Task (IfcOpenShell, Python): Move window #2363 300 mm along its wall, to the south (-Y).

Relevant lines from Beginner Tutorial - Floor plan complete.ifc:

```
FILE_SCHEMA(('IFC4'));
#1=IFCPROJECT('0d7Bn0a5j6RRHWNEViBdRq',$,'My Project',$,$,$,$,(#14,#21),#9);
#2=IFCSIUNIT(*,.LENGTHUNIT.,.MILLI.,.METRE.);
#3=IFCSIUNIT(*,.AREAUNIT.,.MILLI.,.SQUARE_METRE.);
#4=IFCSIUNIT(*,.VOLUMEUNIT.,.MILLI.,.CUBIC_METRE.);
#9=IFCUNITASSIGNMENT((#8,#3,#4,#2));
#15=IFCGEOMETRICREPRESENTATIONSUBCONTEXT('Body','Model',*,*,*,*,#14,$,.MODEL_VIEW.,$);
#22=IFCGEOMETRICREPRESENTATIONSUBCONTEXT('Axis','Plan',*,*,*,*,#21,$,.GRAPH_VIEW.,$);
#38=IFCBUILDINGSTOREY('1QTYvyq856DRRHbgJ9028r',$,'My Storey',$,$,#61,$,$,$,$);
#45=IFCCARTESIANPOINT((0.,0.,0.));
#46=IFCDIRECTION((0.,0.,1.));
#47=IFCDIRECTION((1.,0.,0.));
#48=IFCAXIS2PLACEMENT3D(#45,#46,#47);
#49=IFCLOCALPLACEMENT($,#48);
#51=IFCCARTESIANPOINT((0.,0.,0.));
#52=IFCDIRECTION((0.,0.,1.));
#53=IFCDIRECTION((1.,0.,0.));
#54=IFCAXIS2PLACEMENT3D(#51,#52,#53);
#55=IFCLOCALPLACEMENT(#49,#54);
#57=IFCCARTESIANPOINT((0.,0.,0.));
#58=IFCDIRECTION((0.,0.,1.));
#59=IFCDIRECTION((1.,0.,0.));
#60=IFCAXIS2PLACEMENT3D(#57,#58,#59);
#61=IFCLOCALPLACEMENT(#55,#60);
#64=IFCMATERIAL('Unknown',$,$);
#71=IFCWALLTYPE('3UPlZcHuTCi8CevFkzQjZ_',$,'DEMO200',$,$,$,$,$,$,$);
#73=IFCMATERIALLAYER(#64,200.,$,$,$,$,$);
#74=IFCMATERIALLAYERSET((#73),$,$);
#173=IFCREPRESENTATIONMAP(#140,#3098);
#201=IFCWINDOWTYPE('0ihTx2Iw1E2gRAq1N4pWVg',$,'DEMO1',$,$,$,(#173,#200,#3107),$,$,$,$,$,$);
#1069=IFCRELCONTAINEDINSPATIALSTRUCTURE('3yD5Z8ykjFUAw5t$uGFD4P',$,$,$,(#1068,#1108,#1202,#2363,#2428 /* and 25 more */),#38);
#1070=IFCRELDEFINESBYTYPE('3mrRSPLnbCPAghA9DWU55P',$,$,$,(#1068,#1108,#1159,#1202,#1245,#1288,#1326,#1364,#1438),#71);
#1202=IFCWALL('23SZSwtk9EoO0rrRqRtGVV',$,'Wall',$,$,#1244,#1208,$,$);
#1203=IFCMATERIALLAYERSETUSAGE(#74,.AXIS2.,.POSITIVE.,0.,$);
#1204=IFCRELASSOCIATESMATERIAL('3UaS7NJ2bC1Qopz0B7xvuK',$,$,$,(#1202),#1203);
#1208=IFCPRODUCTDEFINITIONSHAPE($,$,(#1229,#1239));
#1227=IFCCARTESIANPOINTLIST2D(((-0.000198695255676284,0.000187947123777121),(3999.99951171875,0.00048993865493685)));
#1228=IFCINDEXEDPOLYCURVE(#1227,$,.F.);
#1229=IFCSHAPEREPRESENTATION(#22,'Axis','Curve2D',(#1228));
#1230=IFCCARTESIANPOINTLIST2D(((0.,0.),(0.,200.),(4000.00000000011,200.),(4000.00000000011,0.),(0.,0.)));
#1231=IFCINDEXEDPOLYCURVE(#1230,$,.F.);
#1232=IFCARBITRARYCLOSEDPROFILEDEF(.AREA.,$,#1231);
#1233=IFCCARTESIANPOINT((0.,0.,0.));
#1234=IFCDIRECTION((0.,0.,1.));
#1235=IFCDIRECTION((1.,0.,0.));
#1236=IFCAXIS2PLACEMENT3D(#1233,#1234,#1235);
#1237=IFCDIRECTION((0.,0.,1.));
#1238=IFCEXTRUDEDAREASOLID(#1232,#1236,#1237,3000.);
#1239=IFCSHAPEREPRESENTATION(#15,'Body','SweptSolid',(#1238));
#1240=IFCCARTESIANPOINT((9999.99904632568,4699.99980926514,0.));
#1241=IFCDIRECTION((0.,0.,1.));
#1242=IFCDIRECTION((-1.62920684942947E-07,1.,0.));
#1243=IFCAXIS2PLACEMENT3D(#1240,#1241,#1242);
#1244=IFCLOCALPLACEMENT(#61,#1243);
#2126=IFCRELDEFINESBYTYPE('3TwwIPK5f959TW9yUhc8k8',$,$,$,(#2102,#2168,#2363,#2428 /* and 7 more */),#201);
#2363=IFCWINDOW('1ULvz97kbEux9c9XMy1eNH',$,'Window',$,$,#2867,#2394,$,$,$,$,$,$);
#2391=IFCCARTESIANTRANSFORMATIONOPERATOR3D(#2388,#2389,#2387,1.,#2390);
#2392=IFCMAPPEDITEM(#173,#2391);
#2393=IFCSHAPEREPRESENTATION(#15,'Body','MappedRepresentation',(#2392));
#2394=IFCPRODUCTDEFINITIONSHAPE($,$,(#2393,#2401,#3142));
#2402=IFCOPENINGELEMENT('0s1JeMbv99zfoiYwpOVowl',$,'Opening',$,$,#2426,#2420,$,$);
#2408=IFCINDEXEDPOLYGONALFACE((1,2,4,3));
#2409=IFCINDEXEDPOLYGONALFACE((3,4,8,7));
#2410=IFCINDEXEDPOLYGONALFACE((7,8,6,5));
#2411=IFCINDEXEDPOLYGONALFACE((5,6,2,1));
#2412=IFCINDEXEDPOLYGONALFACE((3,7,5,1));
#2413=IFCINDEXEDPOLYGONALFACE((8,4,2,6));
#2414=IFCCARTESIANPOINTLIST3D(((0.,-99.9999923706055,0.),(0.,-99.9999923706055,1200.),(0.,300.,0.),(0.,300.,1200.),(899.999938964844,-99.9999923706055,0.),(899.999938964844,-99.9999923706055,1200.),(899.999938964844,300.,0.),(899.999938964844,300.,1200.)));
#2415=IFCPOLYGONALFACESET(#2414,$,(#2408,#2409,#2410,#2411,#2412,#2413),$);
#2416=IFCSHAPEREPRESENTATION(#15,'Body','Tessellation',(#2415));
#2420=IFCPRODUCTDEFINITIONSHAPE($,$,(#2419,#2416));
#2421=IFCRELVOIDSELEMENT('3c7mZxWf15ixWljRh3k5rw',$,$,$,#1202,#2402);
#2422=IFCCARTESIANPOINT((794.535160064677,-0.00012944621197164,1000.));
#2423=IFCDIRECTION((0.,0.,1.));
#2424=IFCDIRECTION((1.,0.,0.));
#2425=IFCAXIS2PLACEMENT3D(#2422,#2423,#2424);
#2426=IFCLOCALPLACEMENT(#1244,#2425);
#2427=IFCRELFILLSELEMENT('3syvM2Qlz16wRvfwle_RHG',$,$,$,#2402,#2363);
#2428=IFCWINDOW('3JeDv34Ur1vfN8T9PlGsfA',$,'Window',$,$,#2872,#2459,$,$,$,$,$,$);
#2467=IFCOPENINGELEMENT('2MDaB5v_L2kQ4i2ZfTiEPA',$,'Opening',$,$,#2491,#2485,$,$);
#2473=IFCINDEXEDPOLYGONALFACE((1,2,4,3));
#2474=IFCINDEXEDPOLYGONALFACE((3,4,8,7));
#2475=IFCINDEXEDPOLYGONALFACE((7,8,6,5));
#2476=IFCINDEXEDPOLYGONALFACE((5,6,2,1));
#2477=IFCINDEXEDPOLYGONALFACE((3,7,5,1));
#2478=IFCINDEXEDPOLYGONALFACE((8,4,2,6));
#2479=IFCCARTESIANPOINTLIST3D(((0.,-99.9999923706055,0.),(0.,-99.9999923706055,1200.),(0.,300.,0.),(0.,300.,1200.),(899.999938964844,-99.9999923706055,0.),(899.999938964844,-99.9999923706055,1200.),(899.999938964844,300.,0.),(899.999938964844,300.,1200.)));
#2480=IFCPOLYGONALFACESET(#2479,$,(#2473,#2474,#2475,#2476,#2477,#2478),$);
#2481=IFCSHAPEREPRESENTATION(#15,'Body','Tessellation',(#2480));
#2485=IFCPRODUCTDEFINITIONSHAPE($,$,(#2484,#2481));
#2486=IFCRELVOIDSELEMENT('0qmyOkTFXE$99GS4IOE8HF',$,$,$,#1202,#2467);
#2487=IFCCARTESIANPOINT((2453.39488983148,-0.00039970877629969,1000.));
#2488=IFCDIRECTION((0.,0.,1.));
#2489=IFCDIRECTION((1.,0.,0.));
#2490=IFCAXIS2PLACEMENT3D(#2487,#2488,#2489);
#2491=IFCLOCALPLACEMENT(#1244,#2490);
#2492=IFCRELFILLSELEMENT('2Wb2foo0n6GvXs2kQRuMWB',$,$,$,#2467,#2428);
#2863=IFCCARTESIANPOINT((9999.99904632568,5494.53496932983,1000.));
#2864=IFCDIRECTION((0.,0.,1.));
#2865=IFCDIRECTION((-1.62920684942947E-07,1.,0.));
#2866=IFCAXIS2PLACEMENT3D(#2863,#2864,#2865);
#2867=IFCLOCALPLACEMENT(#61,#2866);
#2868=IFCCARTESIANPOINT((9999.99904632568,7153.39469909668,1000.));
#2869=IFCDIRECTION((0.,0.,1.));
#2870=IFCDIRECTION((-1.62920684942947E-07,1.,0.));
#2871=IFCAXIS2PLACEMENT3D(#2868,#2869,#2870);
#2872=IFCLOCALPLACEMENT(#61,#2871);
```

```python
import ifcopenshell
import ifcopenshell.api.geometry
import ifcopenshell.util.placement
import ifcopenshell.util.unit

model = ifcopenshell.open("Beginner Tutorial - Floor plan complete.ifc")
unit_scale = ifcopenshell.util.unit.calculate_unit_scale(model)

window = model.by_guid("1ULvz97kbEux9c9XMy1eNH")
opening = window.FillsVoids[0].RelatingOpeningElement
wall = opening.VoidsElements[0].RelatingBuildingElement

wall_matrix = ifcopenshell.util.placement.get_local_placement(wall.ObjectPlacement)
shift = wall_matrix[:3, 0] * -0.3 / unit_scale
before = ifcopenshell.util.placement.get_local_placement(window.ObjectPlacement)[:3, 3].copy()

# The window is not placed relative to its opening, so move both.
for product in (opening, window):
    matrix = ifcopenshell.util.placement.get_local_placement(product.ObjectPlacement)
    matrix[:3, 3] += shift
    ifcopenshell.api.geometry.edit_object_placement(model, product=product, matrix=matrix, is_si=False)

after = ifcopenshell.util.placement.get_local_placement(window.ObjectPlacement)[:3, 3]
print("window moved by", (after - before).round(3) + 0.0)

model.write("Beginner Tutorial - Floor plan complete-out.ifc")
```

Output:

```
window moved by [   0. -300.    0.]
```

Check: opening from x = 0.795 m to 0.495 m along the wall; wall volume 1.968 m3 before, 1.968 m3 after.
